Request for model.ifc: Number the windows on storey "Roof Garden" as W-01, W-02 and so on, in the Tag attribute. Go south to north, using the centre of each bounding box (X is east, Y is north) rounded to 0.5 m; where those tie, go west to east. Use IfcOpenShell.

First a look at what the model holds.

```python
import ifcopenshell
import ifcopenshell.util.element
import ifcopenshell.util.placement

model = ifcopenshell.open("model.ifc")
print(model.schema)
storey = next(s for s in model.by_type("IfcBuildingStorey") if s.Name == "Roof Garden")
windows = [e for e in ifcopenshell.util.element.get_decomposition(storey) if e.is_a("IfcWindow")]
for e in sorted(windows, key=lambda e: e.id()):
    origin = ifcopenshell.util.placement.get_local_placement(e.ObjectPlacement)[:3, 3]
    print(e.id(), e.Tag, e.Name, origin.round(2) + 0.0, sep=" | ")
```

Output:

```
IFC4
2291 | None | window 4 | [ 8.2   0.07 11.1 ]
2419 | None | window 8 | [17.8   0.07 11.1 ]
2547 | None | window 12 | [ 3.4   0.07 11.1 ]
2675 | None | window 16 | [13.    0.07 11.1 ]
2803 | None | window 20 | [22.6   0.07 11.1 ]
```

```python
import ifcopenshell
import ifcopenshell.geom
import ifcopenshell.util.element
import ifcopenshell.util.shape

model = ifcopenshell.open("model.ifc")
settings = ifcopenshell.geom.settings()
settings.set("use-world-coords", True)


def centre(element):
    shape = ifcopenshell.geom.create_shape(settings, element)
    return ifcopenshell.util.shape.get_bbox_centroid(shape.geometry)


storey = next(s for s in model.by_type("IfcBuildingStorey") if s.Name == "Roof Garden")
windows = [e for e in ifcopenshell.util.element.get_decomposition(storey) if e.is_a("IfcWindow")]

# Insertion points can sit at a corner or the storey origin, so sort by the geometry (in metres).
centres = {e: centre(e) for e in windows}
windows.sort(key=lambda e: (round(centres[e][1] / 0.5), centres[e][0]))

for i, e in enumerate(windows, start=1):
    number = f"W-{i:02d}"
    e.Tag = number
    print(e.id(), number)

model.write("model_rev.ifc")
```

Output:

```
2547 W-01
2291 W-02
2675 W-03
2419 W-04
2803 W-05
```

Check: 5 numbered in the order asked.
